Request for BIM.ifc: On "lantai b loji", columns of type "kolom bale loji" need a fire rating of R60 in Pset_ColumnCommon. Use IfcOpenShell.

First a look at what the model holds.

```python
import ifcopenshell
import ifcopenshell.util.element

model = ifcopenshell.open("BIM.ifc")
print(model.schema)
storey = next(s for s in model.by_type("IfcBuildingStorey") if s.Name == "lantai b loji")
columns = [e for e in ifcopenshell.util.element.get_decomposition(storey) if e.is_a("IfcColumn")]
seen = {}
for e in columns:
    element_type = ifcopenshell.util.element.get_type(e)
    key = (element_type.Name if element_type != e and element_type else None, ifcopenshell.util.element.get_pset(e, "Pset_ColumnCommon", "FireRating"))
    seen[key] = seen.get(key, 0) + 1
for (name, value), count in sorted(seen.items(), key=str):
    print(count, "x", name, "|", value)
```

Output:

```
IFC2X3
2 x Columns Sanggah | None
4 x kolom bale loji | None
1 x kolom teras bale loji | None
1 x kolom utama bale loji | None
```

```python
import ifcopenshell
import ifcopenshell.api.pset
import ifcopenshell.util.element

model = ifcopenshell.open("BIM.ifc")

storey = next(s for s in model.by_type("IfcBuildingStorey") if s.Name == "lantai b loji")
columns = [e for e in ifcopenshell.util.element.get_decomposition(storey) if e.is_a("IfcColumn")]

count = 0
for e in columns:
    element_type = ifcopenshell.util.element.get_type(e)
    if element_type in (None, e) or element_type.Name != "kolom bale loji":
        continue
    # add_pset returns the element's existing set when there is one.
    pset = ifcopenshell.api.pset.add_pset(model, product=e, name="Pset_ColumnCommon")
    ifcopenshell.api.pset.edit_pset(model, pset=pset, properties={"FireRating": "R60"})
    count += 1

print(count, "columns updated")

model.write("BIM_v2.ifc")
```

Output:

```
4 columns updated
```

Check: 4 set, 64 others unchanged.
